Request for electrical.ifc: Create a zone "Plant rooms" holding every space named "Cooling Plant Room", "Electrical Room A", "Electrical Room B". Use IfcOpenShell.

First a look at what the model holds.

```python
import ifcopenshell

model = ifcopenshell.open("electrical.ifc")
print(model.schema)
seen = {}
for space in model.by_type("IfcSpace"):
    seen[space.LongName] = seen.get(space.LongName, 0) + 1
for name, count in sorted(seen.items(), key=str):
    print(count, "x", name)
print("zones:", [z.Name for z in model.by_type("IfcZone")][:20])
```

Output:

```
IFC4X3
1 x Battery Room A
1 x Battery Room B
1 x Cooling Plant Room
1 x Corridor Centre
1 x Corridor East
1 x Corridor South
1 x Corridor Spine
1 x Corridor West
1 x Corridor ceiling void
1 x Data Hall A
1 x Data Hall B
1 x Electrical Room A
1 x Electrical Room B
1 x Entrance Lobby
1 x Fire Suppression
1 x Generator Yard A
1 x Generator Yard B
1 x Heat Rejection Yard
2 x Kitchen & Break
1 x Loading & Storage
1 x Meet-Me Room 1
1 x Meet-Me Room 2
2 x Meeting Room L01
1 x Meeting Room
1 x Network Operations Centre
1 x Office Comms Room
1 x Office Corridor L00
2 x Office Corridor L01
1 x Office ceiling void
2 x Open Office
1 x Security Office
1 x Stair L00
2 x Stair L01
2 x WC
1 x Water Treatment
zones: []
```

```python
import ifcopenshell
import ifcopenshell.api.group
import ifcopenshell.api.root

model = ifcopenshell.open("electrical.ifc")

names = {"Cooling Plant Room", "Electrical Room A", "Electrical Room B"}
spaces = [s for s in model.by_type("IfcSpace") if s.LongName in names]

zone = ifcopenshell.api.root.create_entity(model, ifc_class="IfcZone", name="Plant rooms")
ifcopenshell.api.group.assign_group(model, products=spaces, group=zone)
print(len(spaces), "spaces in", zone.Name)

model.write("electrical_v2.ifc")
```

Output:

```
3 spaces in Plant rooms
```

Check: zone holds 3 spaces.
